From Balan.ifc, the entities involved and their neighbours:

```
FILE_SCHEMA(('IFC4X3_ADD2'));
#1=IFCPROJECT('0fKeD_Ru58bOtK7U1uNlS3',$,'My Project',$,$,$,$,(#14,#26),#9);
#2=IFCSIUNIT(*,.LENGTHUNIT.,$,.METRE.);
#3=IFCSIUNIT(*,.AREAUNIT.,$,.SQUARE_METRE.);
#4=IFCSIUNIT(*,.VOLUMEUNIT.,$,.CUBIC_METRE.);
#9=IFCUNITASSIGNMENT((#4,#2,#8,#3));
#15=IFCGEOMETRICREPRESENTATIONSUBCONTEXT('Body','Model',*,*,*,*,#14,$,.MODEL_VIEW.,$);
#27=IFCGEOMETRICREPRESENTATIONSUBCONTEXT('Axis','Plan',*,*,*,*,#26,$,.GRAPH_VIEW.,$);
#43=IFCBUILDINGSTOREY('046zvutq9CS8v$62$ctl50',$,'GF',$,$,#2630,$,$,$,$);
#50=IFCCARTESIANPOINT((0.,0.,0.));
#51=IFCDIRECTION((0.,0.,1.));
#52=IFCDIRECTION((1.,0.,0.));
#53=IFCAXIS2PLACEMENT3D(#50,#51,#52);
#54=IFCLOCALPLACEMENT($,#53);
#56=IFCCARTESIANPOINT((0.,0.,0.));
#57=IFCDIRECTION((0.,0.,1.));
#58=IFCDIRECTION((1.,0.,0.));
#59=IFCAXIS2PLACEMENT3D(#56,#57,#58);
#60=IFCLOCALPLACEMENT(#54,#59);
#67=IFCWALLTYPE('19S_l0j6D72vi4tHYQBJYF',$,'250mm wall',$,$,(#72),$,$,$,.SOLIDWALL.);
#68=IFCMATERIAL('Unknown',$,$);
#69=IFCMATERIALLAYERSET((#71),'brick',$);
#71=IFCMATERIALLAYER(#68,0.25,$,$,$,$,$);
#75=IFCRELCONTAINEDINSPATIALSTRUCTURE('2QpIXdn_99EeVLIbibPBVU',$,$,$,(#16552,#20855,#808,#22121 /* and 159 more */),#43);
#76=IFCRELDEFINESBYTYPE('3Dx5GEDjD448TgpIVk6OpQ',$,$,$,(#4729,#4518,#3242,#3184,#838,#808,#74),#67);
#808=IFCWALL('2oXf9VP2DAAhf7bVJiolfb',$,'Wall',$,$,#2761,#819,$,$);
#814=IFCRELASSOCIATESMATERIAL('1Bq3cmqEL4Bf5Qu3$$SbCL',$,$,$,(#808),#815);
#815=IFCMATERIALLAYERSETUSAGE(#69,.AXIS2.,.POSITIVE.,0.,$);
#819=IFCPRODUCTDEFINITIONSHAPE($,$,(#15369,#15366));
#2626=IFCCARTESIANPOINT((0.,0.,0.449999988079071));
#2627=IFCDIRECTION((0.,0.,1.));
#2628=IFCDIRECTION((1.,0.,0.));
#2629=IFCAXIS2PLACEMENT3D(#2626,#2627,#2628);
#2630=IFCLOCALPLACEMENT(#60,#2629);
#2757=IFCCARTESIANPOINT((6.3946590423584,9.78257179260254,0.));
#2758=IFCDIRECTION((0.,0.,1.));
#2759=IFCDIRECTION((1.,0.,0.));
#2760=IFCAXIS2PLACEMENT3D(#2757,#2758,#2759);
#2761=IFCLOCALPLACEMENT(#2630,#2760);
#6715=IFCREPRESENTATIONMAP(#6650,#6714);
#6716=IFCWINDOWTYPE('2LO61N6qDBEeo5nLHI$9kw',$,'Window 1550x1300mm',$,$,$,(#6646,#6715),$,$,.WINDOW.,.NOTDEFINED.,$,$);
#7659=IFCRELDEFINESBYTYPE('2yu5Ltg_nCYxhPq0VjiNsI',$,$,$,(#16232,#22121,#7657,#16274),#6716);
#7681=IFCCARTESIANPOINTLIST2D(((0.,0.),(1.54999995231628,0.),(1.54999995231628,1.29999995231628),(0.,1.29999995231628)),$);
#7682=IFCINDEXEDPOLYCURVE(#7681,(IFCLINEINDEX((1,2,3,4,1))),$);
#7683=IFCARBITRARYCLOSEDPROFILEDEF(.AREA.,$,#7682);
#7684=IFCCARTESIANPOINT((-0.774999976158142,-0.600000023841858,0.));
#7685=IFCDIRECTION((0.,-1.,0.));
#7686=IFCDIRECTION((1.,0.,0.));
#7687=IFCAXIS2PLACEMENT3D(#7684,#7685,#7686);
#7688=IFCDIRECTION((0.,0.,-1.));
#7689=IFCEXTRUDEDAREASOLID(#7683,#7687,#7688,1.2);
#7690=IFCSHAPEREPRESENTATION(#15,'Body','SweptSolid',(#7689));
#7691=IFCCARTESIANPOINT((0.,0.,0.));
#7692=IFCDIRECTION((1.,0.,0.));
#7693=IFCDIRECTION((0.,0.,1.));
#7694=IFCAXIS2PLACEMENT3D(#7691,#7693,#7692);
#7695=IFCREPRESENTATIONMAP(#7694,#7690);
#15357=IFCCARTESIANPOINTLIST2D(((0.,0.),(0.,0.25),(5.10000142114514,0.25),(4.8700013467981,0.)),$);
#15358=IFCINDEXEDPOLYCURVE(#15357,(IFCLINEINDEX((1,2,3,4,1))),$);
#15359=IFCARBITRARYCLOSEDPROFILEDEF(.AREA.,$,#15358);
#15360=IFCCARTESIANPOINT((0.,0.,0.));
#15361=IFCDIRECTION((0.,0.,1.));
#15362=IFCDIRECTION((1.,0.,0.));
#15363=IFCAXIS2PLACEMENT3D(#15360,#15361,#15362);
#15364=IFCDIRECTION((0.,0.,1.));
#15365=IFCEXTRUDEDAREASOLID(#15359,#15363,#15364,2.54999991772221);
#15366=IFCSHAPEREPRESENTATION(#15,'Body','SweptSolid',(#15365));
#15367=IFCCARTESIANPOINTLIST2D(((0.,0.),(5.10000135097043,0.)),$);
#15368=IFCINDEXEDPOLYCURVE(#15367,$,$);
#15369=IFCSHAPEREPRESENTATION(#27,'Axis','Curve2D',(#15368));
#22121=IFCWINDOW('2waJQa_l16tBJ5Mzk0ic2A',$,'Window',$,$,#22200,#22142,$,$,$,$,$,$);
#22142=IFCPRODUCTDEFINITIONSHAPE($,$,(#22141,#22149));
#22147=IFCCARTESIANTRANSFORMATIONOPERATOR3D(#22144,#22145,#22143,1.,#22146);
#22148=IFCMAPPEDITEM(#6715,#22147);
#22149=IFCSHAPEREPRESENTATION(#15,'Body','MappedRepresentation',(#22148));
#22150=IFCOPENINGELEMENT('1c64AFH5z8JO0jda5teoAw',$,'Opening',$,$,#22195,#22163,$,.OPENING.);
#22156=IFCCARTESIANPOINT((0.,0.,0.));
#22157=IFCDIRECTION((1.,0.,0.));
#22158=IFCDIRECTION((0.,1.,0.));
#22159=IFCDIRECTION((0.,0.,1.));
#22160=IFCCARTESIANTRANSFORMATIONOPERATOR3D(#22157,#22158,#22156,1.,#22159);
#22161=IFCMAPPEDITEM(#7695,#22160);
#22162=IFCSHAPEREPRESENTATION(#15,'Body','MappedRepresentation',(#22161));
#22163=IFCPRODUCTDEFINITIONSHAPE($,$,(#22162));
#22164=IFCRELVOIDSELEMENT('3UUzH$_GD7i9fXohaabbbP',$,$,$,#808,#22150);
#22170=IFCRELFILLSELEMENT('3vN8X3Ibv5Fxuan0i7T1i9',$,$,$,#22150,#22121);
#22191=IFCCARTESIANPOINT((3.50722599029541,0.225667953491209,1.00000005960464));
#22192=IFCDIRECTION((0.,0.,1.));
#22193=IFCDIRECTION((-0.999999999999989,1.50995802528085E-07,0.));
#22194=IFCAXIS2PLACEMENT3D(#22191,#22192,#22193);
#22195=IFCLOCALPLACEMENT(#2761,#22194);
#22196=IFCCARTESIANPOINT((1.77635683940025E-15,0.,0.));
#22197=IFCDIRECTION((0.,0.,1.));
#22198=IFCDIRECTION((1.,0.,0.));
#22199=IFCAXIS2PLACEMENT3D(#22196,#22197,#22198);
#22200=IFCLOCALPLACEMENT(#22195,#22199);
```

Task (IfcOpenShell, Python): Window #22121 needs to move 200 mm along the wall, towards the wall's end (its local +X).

```python
import ifcopenshell
import ifcopenshell.api.geometry
import ifcopenshell.util.placement

model = ifcopenshell.open("Balan.ifc")

window = model.by_id(22121)
opening = window.FillsVoids[0].RelatingOpeningElement
wall = opening.VoidsElements[0].RelatingBuildingElement

wall_matrix = ifcopenshell.util.placement.get_local_placement(wall.ObjectPlacement)
shift = wall_matrix[:3, 0] * 0.2
before = ifcopenshell.util.placement.get_local_placement(window.ObjectPlacement)[:3, 3].copy()

# The window is placed relative to its opening, so it follows when the opening moves.
matrix = ifcopenshell.util.placement.get_local_placement(opening.ObjectPlacement)
matrix[:3, 3] += shift
ifcopenshell.api.geometry.edit_object_placement(
    model, product=opening, matrix=matrix, is_si=False, should_transform_children=True
)

after = ifcopenshell.util.placement.get_local_placement(window.ObjectPlacement)[:3, 3]
print("window moved by", (after - before).round(3) + 0.0)

model.write("Balan_rev.ifc")
```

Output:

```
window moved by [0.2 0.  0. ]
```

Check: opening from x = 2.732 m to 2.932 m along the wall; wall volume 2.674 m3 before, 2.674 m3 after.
